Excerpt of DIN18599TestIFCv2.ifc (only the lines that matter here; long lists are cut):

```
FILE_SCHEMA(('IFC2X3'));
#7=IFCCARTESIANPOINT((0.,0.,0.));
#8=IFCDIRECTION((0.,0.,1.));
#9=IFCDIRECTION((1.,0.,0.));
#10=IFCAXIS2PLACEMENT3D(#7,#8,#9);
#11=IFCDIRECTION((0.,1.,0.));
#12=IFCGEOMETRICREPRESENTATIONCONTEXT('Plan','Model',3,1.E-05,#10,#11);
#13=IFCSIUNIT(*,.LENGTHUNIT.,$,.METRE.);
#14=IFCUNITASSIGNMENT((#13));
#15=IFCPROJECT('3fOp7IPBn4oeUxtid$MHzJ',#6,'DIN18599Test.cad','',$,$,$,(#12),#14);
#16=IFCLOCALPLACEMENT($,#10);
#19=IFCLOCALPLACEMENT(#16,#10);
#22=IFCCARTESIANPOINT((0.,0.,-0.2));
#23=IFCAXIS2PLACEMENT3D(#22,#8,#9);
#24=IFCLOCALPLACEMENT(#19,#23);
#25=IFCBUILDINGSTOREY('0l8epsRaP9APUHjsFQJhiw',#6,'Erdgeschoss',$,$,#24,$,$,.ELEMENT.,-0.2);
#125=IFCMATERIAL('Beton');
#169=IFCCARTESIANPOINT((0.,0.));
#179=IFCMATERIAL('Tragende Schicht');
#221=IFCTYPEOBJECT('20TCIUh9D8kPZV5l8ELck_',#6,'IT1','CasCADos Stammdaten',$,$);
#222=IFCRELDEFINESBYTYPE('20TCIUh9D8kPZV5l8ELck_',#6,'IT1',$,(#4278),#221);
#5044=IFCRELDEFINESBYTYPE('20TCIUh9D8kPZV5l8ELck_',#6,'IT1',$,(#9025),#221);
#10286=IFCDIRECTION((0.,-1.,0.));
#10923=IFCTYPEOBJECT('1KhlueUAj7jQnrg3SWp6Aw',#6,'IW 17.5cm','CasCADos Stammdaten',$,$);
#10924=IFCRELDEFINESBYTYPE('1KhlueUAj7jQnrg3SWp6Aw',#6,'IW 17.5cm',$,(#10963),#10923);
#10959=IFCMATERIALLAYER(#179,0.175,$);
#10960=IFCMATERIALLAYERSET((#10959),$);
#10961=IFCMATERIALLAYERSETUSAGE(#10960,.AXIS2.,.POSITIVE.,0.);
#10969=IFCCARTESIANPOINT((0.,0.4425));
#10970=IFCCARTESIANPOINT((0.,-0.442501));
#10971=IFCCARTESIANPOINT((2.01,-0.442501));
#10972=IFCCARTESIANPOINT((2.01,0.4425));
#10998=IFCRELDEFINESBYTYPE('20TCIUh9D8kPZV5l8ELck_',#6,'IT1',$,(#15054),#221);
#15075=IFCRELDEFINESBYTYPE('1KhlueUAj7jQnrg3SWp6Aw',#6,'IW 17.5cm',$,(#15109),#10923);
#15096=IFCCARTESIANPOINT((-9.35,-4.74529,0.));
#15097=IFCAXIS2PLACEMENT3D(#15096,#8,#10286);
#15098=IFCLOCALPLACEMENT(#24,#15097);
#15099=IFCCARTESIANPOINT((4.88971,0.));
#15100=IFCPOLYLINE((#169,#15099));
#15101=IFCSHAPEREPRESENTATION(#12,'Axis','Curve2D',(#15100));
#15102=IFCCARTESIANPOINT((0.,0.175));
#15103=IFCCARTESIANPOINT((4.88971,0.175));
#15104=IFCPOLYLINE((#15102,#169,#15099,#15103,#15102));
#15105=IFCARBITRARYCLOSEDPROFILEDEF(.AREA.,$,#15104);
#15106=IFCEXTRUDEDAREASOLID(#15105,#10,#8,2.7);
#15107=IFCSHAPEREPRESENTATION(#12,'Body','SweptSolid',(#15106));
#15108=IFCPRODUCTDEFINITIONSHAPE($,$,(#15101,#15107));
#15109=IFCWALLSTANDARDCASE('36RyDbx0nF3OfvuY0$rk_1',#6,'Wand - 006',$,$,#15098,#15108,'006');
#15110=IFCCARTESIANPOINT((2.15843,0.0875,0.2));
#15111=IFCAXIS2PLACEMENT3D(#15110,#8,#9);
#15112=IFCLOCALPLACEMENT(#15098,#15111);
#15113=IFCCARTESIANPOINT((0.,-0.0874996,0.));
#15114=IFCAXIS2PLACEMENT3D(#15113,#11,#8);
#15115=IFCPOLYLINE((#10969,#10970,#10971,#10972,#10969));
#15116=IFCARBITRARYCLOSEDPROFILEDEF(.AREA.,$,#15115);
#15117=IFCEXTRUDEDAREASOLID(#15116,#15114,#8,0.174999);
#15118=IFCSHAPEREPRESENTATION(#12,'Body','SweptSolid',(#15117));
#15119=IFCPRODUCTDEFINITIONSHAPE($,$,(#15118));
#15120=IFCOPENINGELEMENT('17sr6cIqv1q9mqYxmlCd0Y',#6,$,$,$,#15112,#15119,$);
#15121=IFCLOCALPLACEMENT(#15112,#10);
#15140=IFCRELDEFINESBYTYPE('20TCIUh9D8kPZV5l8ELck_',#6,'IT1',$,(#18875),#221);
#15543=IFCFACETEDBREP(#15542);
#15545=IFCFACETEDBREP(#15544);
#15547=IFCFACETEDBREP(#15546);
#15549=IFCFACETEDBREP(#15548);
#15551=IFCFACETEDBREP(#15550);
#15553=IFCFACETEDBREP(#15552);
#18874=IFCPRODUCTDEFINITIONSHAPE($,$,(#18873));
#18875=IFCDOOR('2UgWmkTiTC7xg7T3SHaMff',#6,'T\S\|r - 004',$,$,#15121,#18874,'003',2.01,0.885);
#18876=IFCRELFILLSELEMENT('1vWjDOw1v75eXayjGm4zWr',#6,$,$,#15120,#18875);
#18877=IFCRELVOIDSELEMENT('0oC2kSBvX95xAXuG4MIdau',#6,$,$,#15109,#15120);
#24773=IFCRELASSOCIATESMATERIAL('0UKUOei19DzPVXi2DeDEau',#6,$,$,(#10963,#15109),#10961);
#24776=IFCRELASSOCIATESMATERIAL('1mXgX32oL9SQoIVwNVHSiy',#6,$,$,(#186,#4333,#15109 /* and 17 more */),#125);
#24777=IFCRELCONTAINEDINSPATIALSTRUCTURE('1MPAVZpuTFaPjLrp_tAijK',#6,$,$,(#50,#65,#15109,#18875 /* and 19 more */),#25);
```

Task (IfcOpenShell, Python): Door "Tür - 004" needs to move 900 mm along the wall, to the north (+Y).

```python
import ifcopenshell
import ifcopenshell.api.geometry
import ifcopenshell.util.placement
import ifcopenshell.util.unit

model = ifcopenshell.open("DIN18599TestIFCv2.ifc")
unit_scale = ifcopenshell.util.unit.calculate_unit_scale(model)

door = model.by_guid("2UgWmkTiTC7xg7T3SHaMff")
opening = door.FillsVoids[0].RelatingOpeningElement
wall = opening.VoidsElements[0].RelatingBuildingElement

wall_matrix = ifcopenshell.util.placement.get_local_placement(wall.ObjectPlacement)
shift = wall_matrix[:3, 0] * -0.9 / unit_scale
before = ifcopenshell.util.placement.get_local_placement(door.ObjectPlacement)[:3, 3].copy()

# The door is placed relative to its opening, so it follows when the opening moves.
matrix = ifcopenshell.util.placement.get_local_placement(opening.ObjectPlacement)
matrix[:3, 3] += shift
ifcopenshell.api.geometry.edit_object_placement(
    model, product=opening, matrix=matrix, is_si=False, should_transform_children=True
)

after = ifcopenshell.util.placement.get_local_placement(door.ObjectPlacement)[:3, 3]
print("door moved by", (after - before).round(3) + 0.0)

model.write("DIN18599TestIFCv2_rev.ifc")
```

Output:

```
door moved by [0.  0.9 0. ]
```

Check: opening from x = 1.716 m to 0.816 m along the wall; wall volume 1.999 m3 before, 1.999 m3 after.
